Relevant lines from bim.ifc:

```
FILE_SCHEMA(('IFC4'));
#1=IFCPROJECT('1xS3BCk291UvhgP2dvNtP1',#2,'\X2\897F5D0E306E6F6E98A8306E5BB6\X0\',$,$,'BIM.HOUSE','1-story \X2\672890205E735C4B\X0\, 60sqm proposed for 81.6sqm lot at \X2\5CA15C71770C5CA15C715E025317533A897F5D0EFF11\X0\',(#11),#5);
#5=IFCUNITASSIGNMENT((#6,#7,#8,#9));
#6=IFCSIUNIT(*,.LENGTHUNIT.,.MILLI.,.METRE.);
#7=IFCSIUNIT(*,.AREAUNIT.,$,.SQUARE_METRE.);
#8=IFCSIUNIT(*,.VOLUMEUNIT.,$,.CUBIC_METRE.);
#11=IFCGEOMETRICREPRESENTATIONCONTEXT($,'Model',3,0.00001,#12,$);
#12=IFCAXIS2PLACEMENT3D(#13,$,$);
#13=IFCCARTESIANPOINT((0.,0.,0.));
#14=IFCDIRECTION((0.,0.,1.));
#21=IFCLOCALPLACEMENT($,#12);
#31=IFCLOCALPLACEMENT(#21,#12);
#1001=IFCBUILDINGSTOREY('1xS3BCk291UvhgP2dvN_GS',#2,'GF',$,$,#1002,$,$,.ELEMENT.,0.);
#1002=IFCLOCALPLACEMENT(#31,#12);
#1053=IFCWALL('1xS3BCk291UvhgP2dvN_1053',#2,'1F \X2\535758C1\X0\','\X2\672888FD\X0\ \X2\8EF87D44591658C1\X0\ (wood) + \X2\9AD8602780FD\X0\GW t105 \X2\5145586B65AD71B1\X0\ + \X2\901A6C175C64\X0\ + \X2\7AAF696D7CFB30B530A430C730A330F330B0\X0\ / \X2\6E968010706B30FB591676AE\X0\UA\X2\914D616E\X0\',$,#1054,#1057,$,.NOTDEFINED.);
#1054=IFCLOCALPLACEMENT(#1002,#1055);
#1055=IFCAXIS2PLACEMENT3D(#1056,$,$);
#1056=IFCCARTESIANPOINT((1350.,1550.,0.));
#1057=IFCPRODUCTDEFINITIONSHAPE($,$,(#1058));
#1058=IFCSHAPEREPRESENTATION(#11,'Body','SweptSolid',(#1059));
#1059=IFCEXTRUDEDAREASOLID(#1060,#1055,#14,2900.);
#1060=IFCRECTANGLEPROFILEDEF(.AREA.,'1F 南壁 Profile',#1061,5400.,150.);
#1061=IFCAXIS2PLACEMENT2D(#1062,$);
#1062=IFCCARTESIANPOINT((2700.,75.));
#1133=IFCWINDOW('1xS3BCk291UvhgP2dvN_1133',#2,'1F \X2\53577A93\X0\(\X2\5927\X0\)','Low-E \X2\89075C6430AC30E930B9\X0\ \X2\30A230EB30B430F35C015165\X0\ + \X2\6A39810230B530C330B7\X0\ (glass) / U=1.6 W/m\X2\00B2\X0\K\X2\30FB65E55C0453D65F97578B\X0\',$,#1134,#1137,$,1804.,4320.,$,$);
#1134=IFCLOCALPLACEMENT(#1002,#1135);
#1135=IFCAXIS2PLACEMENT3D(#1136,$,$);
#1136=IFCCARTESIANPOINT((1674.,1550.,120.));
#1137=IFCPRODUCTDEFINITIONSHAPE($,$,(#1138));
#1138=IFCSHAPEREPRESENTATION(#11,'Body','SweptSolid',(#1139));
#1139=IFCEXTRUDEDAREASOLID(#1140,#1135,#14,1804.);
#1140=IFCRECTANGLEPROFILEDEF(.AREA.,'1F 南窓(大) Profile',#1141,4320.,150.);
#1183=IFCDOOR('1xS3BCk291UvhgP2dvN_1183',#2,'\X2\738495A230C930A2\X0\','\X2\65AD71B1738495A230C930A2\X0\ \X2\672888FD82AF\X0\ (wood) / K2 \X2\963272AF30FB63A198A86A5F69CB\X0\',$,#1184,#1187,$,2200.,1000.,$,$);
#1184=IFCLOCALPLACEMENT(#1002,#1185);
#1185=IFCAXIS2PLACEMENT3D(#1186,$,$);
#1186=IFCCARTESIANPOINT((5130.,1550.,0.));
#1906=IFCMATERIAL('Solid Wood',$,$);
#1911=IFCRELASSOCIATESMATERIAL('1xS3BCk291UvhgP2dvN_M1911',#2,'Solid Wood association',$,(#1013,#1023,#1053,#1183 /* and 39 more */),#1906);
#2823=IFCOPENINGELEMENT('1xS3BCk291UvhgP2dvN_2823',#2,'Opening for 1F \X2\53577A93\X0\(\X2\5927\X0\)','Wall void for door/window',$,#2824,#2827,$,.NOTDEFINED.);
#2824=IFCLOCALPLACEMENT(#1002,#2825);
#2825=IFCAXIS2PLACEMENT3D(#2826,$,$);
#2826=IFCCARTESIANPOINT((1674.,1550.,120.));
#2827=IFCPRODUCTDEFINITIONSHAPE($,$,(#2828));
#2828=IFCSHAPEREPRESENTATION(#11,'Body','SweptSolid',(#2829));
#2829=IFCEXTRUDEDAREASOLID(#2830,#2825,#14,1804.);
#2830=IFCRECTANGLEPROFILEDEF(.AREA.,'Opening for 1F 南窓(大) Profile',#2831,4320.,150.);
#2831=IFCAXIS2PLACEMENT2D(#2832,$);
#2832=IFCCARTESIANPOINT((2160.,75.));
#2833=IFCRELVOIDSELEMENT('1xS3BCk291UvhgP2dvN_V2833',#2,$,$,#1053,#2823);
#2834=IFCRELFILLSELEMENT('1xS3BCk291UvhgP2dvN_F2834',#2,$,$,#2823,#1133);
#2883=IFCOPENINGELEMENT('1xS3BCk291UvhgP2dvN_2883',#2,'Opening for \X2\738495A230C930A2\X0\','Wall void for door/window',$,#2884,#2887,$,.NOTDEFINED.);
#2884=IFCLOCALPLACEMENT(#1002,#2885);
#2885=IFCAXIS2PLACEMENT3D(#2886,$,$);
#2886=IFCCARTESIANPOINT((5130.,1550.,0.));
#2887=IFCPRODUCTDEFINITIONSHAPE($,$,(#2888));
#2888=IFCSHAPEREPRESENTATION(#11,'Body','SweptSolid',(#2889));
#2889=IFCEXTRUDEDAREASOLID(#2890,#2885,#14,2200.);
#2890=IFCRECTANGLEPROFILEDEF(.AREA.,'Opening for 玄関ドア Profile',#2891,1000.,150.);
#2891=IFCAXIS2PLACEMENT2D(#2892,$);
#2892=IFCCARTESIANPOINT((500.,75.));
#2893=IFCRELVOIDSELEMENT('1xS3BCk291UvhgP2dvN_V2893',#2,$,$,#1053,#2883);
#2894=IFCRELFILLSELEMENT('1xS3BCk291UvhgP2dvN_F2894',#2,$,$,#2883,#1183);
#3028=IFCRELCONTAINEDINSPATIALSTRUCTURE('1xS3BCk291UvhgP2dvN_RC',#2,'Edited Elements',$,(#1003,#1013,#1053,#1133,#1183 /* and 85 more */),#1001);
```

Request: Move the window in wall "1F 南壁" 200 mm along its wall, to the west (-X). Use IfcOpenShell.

```python
import ifcopenshell
import ifcopenshell.api.geometry
import ifcopenshell.util.placement
import ifcopenshell.util.unit

model = ifcopenshell.open("bim.ifc")
unit_scale = ifcopenshell.util.unit.calculate_unit_scale(model)

window = model.by_guid("1xS3BCk291UvhgP2dvN_1133")
opening = window.FillsVoids[0].RelatingOpeningElement
wall = opening.VoidsElements[0].RelatingBuildingElement

wall_matrix = ifcopenshell.util.placement.get_local_placement(wall.ObjectPlacement)
shift = wall_matrix[:3, 0] * -0.2 / unit_scale
before = ifcopenshell.util.placement.get_local_placement(window.ObjectPlacement)[:3, 3].copy()

# The window is not placed relative to its opening, so move both.
for product in (opening, window):
    matrix = ifcopenshell.util.placement.get_local_placement(product.ObjectPlacement)
    matrix[:3, 3] += shift
    ifcopenshell.api.geometry.edit_object_placement(model, product=product, matrix=matrix, is_si=False)

after = ifcopenshell.util.placement.get_local_placement(window.ObjectPlacement)[:3, 3]
print("window moved by", (after - before).round(3) + 0.0)

model.write("bim_rev.ifc")
```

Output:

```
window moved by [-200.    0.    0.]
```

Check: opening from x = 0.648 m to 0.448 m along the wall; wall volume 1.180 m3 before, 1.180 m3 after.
